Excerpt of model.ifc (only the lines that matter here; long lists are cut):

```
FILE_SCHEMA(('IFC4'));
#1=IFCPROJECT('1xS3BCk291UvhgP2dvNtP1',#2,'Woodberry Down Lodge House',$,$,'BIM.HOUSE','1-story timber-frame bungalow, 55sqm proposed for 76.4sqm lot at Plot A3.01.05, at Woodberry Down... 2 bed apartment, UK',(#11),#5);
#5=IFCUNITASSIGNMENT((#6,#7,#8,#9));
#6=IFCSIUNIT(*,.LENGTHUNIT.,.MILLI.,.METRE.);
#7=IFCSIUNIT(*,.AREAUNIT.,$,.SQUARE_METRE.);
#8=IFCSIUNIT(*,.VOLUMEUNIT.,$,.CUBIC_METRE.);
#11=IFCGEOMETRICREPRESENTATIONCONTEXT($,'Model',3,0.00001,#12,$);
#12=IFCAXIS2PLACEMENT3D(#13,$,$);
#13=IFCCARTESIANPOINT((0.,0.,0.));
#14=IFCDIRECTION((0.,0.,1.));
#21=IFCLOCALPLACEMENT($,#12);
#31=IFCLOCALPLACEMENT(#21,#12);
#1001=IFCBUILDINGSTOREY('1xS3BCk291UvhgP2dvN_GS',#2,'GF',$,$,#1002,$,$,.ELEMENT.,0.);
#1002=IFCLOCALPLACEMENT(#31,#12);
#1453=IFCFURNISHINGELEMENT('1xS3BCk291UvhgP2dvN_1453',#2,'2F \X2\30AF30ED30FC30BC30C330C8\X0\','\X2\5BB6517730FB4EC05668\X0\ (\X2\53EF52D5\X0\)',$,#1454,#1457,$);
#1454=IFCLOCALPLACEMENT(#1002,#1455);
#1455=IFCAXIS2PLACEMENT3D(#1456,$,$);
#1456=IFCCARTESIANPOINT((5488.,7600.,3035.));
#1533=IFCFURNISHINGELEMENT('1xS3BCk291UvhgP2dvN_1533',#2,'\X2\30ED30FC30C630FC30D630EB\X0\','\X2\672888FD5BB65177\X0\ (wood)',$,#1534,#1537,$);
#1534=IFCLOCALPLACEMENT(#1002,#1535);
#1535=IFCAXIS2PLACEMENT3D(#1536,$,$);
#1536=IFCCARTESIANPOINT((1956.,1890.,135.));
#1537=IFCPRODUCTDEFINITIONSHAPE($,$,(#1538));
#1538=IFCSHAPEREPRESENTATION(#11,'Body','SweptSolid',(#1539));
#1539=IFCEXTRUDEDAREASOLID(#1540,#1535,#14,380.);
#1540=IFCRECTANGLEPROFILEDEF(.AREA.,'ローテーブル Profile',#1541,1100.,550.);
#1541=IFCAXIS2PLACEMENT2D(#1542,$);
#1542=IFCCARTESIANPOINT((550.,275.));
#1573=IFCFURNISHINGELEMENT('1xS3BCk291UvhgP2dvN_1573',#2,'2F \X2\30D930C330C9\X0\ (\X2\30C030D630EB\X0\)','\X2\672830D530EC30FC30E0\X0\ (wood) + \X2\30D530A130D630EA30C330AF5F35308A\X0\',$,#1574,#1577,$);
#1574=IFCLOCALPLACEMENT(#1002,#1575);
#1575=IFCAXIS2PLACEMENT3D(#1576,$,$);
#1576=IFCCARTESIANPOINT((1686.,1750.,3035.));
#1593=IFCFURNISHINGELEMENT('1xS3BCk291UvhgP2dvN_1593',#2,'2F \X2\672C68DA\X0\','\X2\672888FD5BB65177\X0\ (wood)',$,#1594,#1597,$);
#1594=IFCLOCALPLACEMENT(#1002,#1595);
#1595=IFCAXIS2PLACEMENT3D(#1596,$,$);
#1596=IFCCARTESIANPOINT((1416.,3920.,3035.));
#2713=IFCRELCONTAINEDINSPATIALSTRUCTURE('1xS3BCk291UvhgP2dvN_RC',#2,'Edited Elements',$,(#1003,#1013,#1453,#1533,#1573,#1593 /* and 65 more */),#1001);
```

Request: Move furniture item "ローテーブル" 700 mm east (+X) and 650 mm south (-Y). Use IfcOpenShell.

```python
import ifcopenshell
import ifcopenshell.api.geometry
import ifcopenshell.util.placement
import ifcopenshell.util.unit

model = ifcopenshell.open("model.ifc")
unit_scale = ifcopenshell.util.unit.calculate_unit_scale(model)

item = model.by_guid("1xS3BCk291UvhgP2dvN_1533")
matrix = ifcopenshell.util.placement.get_local_placement(item.ObjectPlacement)
matrix[0, 3] += 0.7 / unit_scale
matrix[1, 3] -= 0.65 / unit_scale
ifcopenshell.api.geometry.edit_object_placement(model, product=item, matrix=matrix, is_si=False)

print(ifcopenshell.util.placement.get_local_placement(item.ObjectPlacement).round(3) + 0.0)

model.write("model_updated.ifc")
```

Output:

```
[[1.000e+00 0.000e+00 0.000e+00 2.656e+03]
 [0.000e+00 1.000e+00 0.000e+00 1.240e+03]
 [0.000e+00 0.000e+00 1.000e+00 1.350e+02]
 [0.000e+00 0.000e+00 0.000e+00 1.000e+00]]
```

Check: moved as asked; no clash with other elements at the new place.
